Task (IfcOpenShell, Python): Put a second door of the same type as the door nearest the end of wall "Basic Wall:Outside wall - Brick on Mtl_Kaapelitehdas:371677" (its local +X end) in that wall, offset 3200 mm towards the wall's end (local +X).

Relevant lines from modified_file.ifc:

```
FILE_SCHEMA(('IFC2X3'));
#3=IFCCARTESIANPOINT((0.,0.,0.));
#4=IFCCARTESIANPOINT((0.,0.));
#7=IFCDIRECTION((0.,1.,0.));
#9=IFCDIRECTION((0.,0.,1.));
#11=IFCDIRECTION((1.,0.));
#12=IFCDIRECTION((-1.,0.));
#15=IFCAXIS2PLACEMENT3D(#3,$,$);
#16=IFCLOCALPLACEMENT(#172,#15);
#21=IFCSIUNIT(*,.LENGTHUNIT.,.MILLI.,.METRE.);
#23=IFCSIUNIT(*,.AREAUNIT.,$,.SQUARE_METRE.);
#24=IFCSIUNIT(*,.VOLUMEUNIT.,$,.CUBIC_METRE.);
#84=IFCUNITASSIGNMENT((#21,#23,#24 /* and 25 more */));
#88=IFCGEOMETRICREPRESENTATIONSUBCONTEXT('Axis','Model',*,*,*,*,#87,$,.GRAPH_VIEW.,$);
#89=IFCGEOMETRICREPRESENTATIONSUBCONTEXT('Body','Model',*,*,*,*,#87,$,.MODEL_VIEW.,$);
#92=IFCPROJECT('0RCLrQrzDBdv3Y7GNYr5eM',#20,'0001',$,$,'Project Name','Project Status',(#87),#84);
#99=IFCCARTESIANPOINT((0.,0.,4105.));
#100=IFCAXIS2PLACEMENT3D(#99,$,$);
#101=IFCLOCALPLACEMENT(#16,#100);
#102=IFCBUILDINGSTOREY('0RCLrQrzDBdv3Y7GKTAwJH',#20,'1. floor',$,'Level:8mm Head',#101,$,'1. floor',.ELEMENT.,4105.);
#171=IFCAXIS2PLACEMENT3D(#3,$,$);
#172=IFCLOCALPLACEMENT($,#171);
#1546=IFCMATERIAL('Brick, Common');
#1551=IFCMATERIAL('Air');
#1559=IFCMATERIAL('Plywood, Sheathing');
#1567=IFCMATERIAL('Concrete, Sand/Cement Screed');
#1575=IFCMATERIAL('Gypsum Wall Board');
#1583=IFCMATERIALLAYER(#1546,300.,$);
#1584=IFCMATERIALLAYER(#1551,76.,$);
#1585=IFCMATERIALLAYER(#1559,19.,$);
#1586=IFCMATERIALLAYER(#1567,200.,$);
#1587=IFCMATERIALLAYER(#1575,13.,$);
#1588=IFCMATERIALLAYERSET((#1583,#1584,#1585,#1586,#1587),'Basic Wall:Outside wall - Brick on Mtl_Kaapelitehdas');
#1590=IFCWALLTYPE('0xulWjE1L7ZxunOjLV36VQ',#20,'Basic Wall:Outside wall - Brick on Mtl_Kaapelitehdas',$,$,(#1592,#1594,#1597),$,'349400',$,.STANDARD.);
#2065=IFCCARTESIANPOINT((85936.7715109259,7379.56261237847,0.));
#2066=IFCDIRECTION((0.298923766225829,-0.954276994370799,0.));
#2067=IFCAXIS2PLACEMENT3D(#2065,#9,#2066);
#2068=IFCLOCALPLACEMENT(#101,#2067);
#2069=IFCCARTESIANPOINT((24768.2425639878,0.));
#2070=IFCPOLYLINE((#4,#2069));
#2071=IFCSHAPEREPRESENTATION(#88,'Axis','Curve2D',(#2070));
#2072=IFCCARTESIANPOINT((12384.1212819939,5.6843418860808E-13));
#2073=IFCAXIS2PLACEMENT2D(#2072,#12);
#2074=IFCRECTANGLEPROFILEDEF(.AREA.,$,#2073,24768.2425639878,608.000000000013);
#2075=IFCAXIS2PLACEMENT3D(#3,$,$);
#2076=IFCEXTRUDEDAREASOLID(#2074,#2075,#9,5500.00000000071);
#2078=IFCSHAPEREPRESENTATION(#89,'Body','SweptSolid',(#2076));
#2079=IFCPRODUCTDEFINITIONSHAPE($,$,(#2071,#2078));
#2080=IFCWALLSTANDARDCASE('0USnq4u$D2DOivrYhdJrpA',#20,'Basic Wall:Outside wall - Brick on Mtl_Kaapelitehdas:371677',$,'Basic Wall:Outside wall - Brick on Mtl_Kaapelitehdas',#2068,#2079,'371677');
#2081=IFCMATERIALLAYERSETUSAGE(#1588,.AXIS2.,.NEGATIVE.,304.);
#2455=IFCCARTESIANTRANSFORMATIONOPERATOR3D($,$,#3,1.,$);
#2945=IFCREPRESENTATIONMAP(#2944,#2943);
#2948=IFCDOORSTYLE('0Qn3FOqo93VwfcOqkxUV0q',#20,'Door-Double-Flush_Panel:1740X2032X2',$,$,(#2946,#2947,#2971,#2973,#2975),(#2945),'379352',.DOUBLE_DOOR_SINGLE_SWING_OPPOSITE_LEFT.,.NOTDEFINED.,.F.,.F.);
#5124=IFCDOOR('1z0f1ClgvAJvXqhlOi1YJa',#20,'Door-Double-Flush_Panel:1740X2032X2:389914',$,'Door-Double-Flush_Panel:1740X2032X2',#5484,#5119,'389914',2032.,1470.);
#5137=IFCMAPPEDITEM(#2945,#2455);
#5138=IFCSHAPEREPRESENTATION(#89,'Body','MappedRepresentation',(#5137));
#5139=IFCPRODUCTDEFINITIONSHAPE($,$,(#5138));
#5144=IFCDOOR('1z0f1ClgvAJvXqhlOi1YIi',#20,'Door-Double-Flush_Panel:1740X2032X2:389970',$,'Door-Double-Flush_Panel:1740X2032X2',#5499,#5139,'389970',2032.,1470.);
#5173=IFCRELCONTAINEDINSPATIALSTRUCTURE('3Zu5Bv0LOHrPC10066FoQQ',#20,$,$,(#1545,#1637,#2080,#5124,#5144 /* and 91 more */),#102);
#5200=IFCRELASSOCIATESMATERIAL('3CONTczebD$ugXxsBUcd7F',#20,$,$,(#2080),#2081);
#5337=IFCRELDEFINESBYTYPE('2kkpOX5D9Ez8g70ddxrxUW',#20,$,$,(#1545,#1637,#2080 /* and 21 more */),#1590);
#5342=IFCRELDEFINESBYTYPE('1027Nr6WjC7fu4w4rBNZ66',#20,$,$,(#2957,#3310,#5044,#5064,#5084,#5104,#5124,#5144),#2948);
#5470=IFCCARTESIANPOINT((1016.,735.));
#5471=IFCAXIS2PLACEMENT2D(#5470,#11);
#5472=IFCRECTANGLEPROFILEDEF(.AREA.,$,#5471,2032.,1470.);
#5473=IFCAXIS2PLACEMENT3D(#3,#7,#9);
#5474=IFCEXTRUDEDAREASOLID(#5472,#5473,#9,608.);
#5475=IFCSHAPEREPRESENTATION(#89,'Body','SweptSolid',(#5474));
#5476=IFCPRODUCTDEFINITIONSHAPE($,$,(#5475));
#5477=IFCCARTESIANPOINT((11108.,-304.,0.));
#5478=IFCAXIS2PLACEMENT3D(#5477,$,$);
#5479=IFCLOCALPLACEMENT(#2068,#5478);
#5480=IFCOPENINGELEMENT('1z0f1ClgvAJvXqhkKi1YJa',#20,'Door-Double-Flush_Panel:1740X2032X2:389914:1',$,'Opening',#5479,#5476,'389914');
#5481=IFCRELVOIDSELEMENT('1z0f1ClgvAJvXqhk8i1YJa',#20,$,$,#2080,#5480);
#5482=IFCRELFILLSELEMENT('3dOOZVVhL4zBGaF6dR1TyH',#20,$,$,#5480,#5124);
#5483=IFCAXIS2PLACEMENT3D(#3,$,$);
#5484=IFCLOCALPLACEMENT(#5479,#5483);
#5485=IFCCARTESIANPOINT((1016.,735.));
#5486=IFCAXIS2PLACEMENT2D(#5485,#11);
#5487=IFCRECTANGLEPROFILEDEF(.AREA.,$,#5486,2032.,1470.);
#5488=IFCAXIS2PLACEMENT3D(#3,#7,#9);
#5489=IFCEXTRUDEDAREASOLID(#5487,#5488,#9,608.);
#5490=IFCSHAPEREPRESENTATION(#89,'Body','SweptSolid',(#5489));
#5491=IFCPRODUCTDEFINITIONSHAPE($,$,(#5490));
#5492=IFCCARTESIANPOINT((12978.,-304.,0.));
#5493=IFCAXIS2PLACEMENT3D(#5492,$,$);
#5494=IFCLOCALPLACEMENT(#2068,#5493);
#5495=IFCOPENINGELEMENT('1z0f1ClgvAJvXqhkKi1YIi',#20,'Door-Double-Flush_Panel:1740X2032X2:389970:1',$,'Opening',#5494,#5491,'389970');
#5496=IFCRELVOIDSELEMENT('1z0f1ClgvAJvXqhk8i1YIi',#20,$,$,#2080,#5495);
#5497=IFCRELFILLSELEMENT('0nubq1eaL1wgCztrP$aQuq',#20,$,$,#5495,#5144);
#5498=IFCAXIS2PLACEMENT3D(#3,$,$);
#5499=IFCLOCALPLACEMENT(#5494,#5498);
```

```python
import ifcopenshell
import ifcopenshell.api.feature
import ifcopenshell.api.geometry
import ifcopenshell.api.root
import ifcopenshell.geom
import ifcopenshell.util.element
import ifcopenshell.util.placement
import ifcopenshell.util.shape
import ifcopenshell.util.unit

model = ifcopenshell.open("modified_file.ifc")
unit_scale = ifcopenshell.util.unit.calculate_unit_scale(model)
settings = ifcopenshell.geom.settings()


def volume(element):
    """Net volume in cubic metres, openings subtracted."""
    shape = ifcopenshell.geom.create_shape(settings, element)
    return ifcopenshell.util.shape.get_volume(shape.geometry)


def reuse_history(source, copy):
    """copy_class also copies each property set's owner history, people and application; keep the originals."""
    for rel in copy.IsDefinedBy:
        if rel.is_a("IfcRelDefinesByProperties") and (history := rel.RelatingPropertyDefinition.OwnerHistory):
            rel.RelatingPropertyDefinition.OwnerHistory = source.OwnerHistory
            ifcopenshell.util.element.remove_deep2(model, history)


door = model.by_guid("1z0f1ClgvAJvXqhlOi1YIi")
opening = door.FillsVoids[0].RelatingOpeningElement
wall = opening.VoidsElements[0].RelatingBuildingElement
before = volume(wall)
shift = ifcopenshell.util.placement.get_local_placement(wall.ObjectPlacement)[:3, 0] * 3.2 / unit_scale

# copy_class copies the void relationship, type, container and properties, but no geometry.
new_opening = ifcopenshell.api.root.copy_class(model, product=opening)
new_opening.Representation = ifcopenshell.util.element.copy_deep(
    model, opening.Representation, exclude=["IfcGeometricRepresentationContext", "IfcRepresentationMap"]
)
new_opening.Name = "Door-Double-Flush_Panel:1740X2032X2"
new_opening.Tag = None
new_door = ifcopenshell.api.root.copy_class(model, product=door)
new_door.Representation = ifcopenshell.util.element.copy_deep(
    model, door.Representation, exclude=["IfcGeometricRepresentationContext", "IfcRepresentationMap"]
)
new_door.Name = "Door-Double-Flush_Panel:1740X2032X2"
new_door.Tag = None
reuse_history(door, new_door)
fills = ifcopenshell.api.feature.add_filling(model, opening=new_opening, element=new_door)
fills.OwnerHistory = new_door.OwnerHistory  # required in IFC2X3

for old, new in ((opening, new_opening), (door, new_door)):
    matrix = ifcopenshell.util.placement.get_local_placement(old.ObjectPlacement)
    matrix[:3, 3] += shift
    ifcopenshell.api.geometry.edit_object_placement(model, product=new, matrix=matrix, is_si=False)

after = volume(wall)

print(f"wall volume {before:.3f} -> {after:.3f} m3")

model.write("modified_file_updated.ifc")
```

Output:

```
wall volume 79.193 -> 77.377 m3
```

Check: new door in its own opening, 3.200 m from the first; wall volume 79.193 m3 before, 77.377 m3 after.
